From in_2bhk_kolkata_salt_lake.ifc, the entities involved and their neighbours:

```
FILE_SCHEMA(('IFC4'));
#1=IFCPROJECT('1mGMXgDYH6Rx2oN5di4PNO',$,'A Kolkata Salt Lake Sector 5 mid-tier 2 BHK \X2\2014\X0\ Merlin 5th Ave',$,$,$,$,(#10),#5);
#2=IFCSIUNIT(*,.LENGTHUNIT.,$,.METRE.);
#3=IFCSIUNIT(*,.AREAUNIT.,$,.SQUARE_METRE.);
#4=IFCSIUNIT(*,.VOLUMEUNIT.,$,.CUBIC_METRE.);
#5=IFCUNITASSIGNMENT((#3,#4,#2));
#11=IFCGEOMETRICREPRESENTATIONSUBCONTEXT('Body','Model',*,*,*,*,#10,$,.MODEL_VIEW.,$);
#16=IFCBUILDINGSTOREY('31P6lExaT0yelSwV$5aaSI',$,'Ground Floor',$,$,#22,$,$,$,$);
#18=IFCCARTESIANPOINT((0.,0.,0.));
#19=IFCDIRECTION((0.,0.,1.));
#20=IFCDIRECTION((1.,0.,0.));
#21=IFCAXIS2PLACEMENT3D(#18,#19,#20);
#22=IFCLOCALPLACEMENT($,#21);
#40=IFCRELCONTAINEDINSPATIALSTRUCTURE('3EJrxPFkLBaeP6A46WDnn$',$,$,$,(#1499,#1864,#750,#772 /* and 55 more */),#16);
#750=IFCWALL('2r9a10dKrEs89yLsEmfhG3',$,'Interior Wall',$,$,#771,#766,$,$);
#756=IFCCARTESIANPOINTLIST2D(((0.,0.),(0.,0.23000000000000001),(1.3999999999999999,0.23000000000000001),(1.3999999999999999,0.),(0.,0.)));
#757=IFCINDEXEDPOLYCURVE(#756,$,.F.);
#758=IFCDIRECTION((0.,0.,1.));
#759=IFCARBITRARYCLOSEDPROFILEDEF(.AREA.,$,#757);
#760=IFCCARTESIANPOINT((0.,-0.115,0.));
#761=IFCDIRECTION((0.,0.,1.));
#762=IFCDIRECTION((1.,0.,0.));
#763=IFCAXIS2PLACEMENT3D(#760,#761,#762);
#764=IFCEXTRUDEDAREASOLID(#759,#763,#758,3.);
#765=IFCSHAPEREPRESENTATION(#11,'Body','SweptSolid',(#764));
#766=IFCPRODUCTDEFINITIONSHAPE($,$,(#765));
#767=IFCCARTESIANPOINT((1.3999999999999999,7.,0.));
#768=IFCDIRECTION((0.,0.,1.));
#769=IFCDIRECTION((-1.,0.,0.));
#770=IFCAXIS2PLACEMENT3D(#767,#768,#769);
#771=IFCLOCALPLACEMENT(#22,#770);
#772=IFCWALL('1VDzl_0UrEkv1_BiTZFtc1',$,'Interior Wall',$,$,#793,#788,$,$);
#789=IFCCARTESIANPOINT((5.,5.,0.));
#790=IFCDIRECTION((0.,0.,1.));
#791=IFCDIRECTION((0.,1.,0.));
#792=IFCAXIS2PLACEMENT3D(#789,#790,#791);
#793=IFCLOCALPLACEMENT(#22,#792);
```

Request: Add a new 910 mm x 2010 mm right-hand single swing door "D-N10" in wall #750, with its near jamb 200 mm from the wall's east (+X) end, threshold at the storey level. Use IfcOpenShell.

```python
import numpy as np
import ifcopenshell
import ifcopenshell.api.feature
import ifcopenshell.api.geometry
import ifcopenshell.api.root
import ifcopenshell.api.spatial
import ifcopenshell.geom
import ifcopenshell.util.element
import ifcopenshell.util.placement
import ifcopenshell.util.representation
import ifcopenshell.util.shape
import ifcopenshell.util.unit

model = ifcopenshell.open("in_2bhk_kolkata_salt_lake.ifc")
unit_scale = ifcopenshell.util.unit.calculate_unit_scale(model)
settings = ifcopenshell.geom.settings()


def volume(element):
    """Net volume in cubic metres, openings subtracted."""
    shape = ifcopenshell.geom.create_shape(settings, element)
    return ifcopenshell.util.shape.get_volume(shape.geometry)


wall = model.by_guid("2r9a10dKrEs89yLsEmfhG3")
storey = ifcopenshell.util.element.get_container(wall, ifc_class="IfcBuildingStorey")
context = ifcopenshell.util.representation.get_context(model, "Model", "Body", "MODEL_VIEW")
before = volume(wall)

width, height, from_end, sill = 0.91, 2.01, 0.2, 0.0  # metres

# The wall runs along its own X axis, and the end named is its -X end.
wall_shape = ifcopenshell.geom.create_shape(settings, wall)
x, y, z = ifcopenshell.util.shape.get_vertices(wall_shape.geometry).T
start = x.min() + from_end
face, thickness = float(y.min()), float(y.max() - y.min())
wall_matrix = ifcopenshell.util.placement.get_local_placement(wall.ObjectPlacement)
level = ifcopenshell.util.placement.get_local_placement(storey.ObjectPlacement)[2, 3]


def in_wall(x, y):
    """Placement at x, y metres in the wall's axes, at sill height."""
    matrix = wall_matrix.copy()
    matrix[:, 3] = wall_matrix @ np.array([x / unit_scale, y / unit_scale, 0.0, 1.0])
    matrix[2, 3] = level + sill / unit_scale
    return matrix


# Opening: a box that overshoots both wall faces by 50 mm.
opening = ifcopenshell.api.root.create_entity(model, ifc_class="IfcOpeningElement", predefined_type="OPENING")
box = ifcopenshell.api.geometry.add_wall_representation(
    model, context=context, length=width, height=height, thickness=thickness + 0.1
)
ifcopenshell.api.geometry.assign_representation(model, product=opening, representation=box)
ifcopenshell.api.geometry.edit_object_placement(model, product=opening, matrix=in_wall(start, face - 0.05), is_si=False)
ifcopenshell.api.feature.add_feature(model, feature=opening, element=wall)

door = ifcopenshell.api.root.create_entity(model, ifc_class="IfcDoor", name="D-N10", predefined_type="DOOR")
door.OverallWidth, door.OverallHeight = width / unit_scale, height / unit_scale
door.OperationType = "SINGLE_SWING_RIGHT"
body = ifcopenshell.api.geometry.add_door_representation(
    model,
    context=context,
    overall_width=door.OverallWidth,
    overall_height=door.OverallHeight,
    operation_type="SINGLE_SWING_RIGHT",
    lining_properties={"LiningDepth": thickness / unit_scale, "ThresholdDepth": thickness / unit_scale},
)
ifcopenshell.api.geometry.assign_representation(model, product=door, representation=body)
ifcopenshell.api.spatial.assign_container(model, products=[door], relating_structure=storey)
ifcopenshell.api.feature.add_filling(model, opening=opening, element=door)

# The lining spans the wall, so the door starts at the wall face.
ifcopenshell.api.geometry.edit_object_placement(model, product=door, matrix=in_wall(start, face), is_si=False)

after = volume(wall)

print(f"wall volume {before:.3f} -> {after:.3f} m3")

model.write("in_2bhk_kolkata_salt_lake_edited.ifc")
```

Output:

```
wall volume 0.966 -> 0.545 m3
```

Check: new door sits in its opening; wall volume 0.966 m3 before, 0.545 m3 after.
